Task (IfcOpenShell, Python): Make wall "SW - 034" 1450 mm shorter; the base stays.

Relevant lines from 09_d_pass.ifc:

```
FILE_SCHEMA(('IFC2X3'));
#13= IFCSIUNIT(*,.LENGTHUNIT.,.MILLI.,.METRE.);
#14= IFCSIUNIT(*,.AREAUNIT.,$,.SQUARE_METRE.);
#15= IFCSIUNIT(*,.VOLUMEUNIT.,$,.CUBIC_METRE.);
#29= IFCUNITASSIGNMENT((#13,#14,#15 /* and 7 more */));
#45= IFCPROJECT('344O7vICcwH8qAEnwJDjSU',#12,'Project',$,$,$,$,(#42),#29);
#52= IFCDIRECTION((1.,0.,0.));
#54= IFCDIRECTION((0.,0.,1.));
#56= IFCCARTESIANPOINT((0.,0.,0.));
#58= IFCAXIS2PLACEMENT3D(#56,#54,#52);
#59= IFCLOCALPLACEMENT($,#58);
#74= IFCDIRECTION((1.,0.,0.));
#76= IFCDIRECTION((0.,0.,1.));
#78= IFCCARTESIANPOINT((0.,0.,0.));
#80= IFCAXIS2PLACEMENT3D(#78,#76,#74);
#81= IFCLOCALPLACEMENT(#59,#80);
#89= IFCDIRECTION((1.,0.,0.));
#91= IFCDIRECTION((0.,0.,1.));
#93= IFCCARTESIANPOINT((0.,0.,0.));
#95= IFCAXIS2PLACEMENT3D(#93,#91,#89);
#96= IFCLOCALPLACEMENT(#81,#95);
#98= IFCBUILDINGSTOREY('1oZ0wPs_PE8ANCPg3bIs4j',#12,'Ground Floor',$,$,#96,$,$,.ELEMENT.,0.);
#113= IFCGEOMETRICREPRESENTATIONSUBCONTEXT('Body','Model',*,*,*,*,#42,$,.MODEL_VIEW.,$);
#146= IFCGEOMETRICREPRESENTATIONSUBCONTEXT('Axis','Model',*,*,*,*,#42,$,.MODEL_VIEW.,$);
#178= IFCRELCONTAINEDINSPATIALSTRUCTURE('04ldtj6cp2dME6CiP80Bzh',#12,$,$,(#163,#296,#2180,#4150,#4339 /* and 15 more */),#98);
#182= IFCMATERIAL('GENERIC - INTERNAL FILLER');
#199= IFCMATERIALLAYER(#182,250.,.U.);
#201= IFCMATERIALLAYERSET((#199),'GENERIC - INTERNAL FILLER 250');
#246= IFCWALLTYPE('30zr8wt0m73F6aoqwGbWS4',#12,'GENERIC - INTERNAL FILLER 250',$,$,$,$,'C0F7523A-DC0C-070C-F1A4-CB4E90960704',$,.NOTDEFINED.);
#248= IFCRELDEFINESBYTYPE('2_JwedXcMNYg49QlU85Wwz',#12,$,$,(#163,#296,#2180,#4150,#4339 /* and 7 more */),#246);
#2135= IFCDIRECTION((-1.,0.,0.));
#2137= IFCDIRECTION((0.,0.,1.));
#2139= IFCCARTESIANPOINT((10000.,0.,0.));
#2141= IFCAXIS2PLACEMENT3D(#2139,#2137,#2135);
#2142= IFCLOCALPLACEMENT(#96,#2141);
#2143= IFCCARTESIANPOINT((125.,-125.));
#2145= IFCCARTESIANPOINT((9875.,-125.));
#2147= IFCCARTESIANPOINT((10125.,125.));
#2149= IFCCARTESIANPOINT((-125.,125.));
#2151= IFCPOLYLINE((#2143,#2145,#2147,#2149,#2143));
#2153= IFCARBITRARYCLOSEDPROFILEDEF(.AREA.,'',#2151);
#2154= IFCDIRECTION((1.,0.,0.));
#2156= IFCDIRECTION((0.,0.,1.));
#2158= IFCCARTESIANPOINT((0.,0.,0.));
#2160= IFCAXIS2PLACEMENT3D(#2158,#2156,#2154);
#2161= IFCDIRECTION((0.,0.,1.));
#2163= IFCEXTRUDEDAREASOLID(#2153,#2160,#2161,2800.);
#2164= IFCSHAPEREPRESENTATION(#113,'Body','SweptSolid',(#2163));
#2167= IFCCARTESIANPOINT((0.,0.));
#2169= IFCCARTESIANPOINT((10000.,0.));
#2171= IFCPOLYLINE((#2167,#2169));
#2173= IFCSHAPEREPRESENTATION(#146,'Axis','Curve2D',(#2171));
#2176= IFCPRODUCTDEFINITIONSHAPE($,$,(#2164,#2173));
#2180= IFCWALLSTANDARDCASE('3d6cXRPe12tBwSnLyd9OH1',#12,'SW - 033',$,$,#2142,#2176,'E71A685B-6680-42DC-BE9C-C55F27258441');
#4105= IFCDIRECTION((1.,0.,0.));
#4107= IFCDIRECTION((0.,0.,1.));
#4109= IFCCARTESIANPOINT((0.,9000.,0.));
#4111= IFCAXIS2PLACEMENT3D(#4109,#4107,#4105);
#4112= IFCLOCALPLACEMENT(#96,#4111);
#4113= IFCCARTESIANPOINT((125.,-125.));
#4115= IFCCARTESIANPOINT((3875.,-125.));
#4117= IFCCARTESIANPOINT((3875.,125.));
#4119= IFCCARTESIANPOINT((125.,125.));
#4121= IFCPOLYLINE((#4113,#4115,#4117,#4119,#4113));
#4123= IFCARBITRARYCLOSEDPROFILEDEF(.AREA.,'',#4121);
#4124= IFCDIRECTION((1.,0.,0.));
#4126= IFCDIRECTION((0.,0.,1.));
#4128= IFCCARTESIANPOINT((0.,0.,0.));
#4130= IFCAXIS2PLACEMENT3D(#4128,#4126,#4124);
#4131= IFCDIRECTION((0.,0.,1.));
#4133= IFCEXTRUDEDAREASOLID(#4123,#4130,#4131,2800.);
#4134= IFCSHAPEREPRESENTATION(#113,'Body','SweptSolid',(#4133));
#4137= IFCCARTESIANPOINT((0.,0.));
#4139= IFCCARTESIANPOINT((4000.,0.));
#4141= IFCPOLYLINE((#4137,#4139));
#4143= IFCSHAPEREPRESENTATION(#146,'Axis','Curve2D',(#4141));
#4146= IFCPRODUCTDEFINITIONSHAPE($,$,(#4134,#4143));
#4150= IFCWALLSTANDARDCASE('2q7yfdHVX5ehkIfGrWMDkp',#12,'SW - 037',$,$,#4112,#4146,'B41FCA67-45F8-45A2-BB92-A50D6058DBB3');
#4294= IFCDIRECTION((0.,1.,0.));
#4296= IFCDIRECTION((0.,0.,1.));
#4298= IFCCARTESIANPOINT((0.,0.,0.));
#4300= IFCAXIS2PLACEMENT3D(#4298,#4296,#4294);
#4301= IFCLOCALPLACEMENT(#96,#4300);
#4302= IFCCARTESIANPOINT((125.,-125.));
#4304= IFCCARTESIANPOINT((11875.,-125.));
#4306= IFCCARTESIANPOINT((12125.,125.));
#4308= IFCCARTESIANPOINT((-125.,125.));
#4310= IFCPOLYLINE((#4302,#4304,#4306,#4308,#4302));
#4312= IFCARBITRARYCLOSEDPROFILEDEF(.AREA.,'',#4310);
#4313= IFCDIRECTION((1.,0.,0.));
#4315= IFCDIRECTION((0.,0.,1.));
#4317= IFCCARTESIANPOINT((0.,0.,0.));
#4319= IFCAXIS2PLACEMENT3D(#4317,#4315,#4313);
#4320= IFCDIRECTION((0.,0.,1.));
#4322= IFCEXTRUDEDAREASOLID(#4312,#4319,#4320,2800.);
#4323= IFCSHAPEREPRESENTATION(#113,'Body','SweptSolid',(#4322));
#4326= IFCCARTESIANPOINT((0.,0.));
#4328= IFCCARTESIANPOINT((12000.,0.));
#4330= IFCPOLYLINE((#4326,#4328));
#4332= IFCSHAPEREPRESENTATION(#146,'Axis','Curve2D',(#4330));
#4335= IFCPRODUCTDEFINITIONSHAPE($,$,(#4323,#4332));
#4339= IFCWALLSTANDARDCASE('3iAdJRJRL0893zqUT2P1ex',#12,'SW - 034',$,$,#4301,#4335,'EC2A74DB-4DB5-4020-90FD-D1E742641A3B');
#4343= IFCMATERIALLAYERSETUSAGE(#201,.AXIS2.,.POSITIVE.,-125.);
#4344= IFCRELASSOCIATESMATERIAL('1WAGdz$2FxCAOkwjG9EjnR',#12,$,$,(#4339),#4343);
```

```python
import ifcopenshell
import ifcopenshell.geom
import ifcopenshell.util.representation
import ifcopenshell.util.shape

model = ifcopenshell.open("09_d_pass.ifc")
settings = ifcopenshell.geom.settings()


def volume(element):
    """Net volume in cubic metres, openings subtracted."""
    shape = ifcopenshell.geom.create_shape(settings, element)
    return ifcopenshell.util.shape.get_volume(shape.geometry)


wall = model.by_guid("3iAdJRJRL0893zqUT2P1ex")
before = volume(wall)

body = ifcopenshell.util.representation.get_representation(wall, "Model", "Body")
solid = body.Items[0]
old_height = solid.Depth
solid.Depth -= 1450.0
after = volume(wall)

print(f"height {old_height:g} -> {solid.Depth:g}, volume {before:.3f} -> {after:.3f} m3")

model.write("09_d_pass-out.ifc")
```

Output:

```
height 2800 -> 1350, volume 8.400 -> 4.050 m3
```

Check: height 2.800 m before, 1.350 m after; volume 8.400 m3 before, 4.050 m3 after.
